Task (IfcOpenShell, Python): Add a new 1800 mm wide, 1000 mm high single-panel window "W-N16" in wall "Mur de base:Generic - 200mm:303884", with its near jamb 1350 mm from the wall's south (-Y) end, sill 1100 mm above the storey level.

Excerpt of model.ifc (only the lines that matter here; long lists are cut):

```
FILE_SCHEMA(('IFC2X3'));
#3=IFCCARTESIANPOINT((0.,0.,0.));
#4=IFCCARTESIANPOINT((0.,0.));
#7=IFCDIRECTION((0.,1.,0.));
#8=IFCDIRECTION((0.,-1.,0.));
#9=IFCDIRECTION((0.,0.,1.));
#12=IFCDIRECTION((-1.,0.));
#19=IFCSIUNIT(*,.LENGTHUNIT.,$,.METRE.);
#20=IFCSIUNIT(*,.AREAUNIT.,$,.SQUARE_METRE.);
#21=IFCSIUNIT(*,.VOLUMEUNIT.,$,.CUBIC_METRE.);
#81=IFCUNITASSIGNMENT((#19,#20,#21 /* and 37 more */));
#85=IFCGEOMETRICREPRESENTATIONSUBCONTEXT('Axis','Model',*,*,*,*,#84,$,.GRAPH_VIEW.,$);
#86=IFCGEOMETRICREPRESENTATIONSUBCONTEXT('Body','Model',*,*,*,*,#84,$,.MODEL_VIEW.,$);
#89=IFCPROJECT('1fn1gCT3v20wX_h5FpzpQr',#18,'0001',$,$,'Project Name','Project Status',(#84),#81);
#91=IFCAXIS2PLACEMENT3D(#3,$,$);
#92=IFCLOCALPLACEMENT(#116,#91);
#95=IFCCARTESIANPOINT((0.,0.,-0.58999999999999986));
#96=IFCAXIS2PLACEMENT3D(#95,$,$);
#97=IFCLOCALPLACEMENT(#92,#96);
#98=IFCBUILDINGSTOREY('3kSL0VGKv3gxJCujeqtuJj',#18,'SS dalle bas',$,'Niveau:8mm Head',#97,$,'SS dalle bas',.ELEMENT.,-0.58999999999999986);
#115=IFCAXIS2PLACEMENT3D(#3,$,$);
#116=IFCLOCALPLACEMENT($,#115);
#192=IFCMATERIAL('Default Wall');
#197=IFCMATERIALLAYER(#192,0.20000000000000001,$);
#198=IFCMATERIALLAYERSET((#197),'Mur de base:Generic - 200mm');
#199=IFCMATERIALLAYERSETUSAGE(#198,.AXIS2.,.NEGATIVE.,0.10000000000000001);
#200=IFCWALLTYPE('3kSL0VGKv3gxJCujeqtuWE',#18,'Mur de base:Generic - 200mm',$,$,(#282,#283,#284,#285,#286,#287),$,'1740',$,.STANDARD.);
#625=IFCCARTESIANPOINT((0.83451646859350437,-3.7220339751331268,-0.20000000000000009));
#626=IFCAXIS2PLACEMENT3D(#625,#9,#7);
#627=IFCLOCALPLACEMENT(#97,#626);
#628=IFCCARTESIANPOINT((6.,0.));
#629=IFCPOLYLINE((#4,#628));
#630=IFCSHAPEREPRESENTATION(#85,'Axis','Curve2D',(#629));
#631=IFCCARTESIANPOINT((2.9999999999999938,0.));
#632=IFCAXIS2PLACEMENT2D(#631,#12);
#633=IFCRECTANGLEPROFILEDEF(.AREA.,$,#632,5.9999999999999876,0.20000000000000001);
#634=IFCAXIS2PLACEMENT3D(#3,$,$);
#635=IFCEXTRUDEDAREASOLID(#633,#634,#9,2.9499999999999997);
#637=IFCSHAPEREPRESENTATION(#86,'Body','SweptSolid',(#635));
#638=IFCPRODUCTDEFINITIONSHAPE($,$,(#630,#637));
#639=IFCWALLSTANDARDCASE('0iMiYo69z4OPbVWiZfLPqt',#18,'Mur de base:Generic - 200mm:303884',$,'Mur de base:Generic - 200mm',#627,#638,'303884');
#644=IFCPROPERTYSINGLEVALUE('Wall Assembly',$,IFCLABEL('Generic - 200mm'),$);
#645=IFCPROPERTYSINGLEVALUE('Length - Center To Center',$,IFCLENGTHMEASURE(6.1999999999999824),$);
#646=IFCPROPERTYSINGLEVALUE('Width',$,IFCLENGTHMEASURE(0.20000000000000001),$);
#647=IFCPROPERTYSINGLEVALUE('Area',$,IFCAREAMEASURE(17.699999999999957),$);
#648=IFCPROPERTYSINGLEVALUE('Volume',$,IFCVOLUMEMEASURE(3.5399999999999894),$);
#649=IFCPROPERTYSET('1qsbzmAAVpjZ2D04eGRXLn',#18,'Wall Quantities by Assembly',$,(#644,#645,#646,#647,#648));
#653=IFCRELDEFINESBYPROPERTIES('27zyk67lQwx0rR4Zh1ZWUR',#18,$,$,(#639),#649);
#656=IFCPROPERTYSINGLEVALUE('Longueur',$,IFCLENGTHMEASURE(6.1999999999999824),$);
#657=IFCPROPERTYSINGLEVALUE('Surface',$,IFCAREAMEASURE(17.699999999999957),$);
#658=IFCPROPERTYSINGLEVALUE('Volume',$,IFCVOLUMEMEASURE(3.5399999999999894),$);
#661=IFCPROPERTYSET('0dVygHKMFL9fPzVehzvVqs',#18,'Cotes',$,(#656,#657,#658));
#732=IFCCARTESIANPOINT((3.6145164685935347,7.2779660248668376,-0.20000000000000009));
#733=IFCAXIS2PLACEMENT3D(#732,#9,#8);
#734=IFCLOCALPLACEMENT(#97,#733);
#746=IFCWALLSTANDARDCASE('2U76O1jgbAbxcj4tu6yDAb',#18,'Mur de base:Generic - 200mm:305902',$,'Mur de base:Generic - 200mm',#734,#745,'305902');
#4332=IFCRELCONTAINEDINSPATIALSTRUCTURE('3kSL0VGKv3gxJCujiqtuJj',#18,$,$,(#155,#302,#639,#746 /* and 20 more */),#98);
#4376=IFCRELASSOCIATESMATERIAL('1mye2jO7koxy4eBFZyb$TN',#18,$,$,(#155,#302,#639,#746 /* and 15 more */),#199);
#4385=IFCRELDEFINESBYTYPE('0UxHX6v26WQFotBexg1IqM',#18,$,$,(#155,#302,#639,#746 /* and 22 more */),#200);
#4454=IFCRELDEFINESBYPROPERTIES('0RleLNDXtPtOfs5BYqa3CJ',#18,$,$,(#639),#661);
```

```python
import numpy as np
import ifcopenshell
import ifcopenshell.api.feature
import ifcopenshell.api.geometry
import ifcopenshell.api.pset
import ifcopenshell.api.root
import ifcopenshell.api.spatial
import ifcopenshell.api.type
import ifcopenshell.geom
import ifcopenshell.util.element
import ifcopenshell.util.placement
import ifcopenshell.util.representation
import ifcopenshell.util.shape
import ifcopenshell.util.unit

model = ifcopenshell.open("model.ifc")
unit_scale = ifcopenshell.util.unit.calculate_unit_scale(model)
area_scale = ifcopenshell.util.unit.calculate_unit_scale(model, "AREAUNIT")
volume_scale = ifcopenshell.util.unit.calculate_unit_scale(model, "VOLUMEUNIT")
settings = ifcopenshell.geom.settings()


def volume(element):
    """Net volume in cubic metres, openings subtracted."""
    shape = ifcopenshell.geom.create_shape(settings, element)
    return ifcopenshell.util.shape.get_volume(shape.geometry)


wall = model.by_guid("0iMiYo69z4OPbVWiZfLPqt")
storey = ifcopenshell.util.element.get_container(wall, ifc_class="IfcBuildingStorey")
context = ifcopenshell.util.representation.get_context(model, "Model", "Body", "MODEL_VIEW")
before = volume(wall)

width, height, from_end, sill = 1.8, 1, 1.35, 1.1  # metres

# The wall runs along its own X axis, and the end named is its -X end.
wall_shape = ifcopenshell.geom.create_shape(settings, wall)
x, y, z = ifcopenshell.util.shape.get_vertices(wall_shape.geometry).T
start = x.min() + from_end
face, thickness = float(y.min()), float(y.max() - y.min())
wall_matrix = ifcopenshell.util.placement.get_local_placement(wall.ObjectPlacement)
level = ifcopenshell.util.placement.get_local_placement(storey.ObjectPlacement)[2, 3]


def in_wall(x, y):
    """Placement at x, y metres in the wall's axes, at sill height."""
    matrix = wall_matrix.copy()
    matrix[:, 3] = wall_matrix @ np.array([x / unit_scale, y / unit_scale, 0.0, 1.0])
    matrix[2, 3] = level + sill / unit_scale
    return matrix


# Opening: a box that overshoots both wall faces by 50 mm.
opening = ifcopenshell.api.root.create_entity(model, ifc_class="IfcOpeningElement")
box = ifcopenshell.api.geometry.add_wall_representation(
    model, context=context, length=width, height=height, thickness=thickness + 0.1
)
ifcopenshell.api.geometry.assign_representation(model, product=opening, representation=box)
ifcopenshell.api.geometry.edit_object_placement(model, product=opening, matrix=in_wall(start, face - 0.05), is_si=False)
ifcopenshell.api.feature.add_feature(model, feature=opening, element=wall)

window = ifcopenshell.api.root.create_entity(model, ifc_class="IfcWindow", name="W-N16")
window.OverallWidth, window.OverallHeight = width / unit_scale, height / unit_scale
body = ifcopenshell.api.geometry.add_window_representation(
    model,
    context=context,
    overall_width=window.OverallWidth,
    overall_height=window.OverallHeight,
    partition_type="SINGLE_PANEL",
)
ifcopenshell.api.geometry.assign_representation(model, product=window, representation=body)
ifcopenshell.api.spatial.assign_container(model, products=[window], relating_structure=storey)
fills = ifcopenshell.api.feature.add_filling(model, opening=opening, element=window)
fills.OwnerHistory = window.OwnerHistory  # required in IFC2X3

# IFC2X3 keeps the operation on the window style.
style = ifcopenshell.api.root.create_entity(model, ifc_class="IfcWindowStyle", name="W-N16")
style.OperationType, style.ConstructionType = "SINGLE_PANEL", "NOTDEFINED"
style.ParameterTakesPrecedence = style.Sizeable = False
ifcopenshell.api.type.assign_type(model, related_objects=[window], relating_type=style)

# Centre the window in the wall's thickness.
ifcopenshell.api.geometry.edit_object_placement(model, product=window, matrix=in_wall(start, face), is_si=False)
window_shape = ifcopenshell.geom.create_shape(settings, window)
depth = ifcopenshell.util.shape.get_vertices(window_shape.geometry)[:, 1]
offset = face + thickness / 2 - (depth.min() + depth.max()) / 2
ifcopenshell.api.geometry.edit_object_placement(model, product=window, matrix=in_wall(start, offset), is_si=False)

after = volume(wall)

# Update the wall's stored quantities.
pset = model.by_id(ifcopenshell.util.element.get_pset(wall, "Wall Quantities by Assembly", should_inherit=False)["id"])
ifcopenshell.api.pset.edit_pset(model, pset=pset, properties={
    "Area": model.create_entity("IfcAreaMeasure", after / thickness / area_scale),
    "Volume": model.create_entity("IfcVolumeMeasure", after / volume_scale),
})
pset = model.by_id(ifcopenshell.util.element.get_pset(wall, "Cotes", should_inherit=False)["id"])
ifcopenshell.api.pset.edit_pset(model, pset=pset, properties={
    "Surface": model.create_entity("IfcAreaMeasure", after / thickness / area_scale),
    "Volume": model.create_entity("IfcVolumeMeasure", after / volume_scale),
})

print(f"wall volume {before:.3f} -> {after:.3f} m3")

model.write("model-out.ifc")
```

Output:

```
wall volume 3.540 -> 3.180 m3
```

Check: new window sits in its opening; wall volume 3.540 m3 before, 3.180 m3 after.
